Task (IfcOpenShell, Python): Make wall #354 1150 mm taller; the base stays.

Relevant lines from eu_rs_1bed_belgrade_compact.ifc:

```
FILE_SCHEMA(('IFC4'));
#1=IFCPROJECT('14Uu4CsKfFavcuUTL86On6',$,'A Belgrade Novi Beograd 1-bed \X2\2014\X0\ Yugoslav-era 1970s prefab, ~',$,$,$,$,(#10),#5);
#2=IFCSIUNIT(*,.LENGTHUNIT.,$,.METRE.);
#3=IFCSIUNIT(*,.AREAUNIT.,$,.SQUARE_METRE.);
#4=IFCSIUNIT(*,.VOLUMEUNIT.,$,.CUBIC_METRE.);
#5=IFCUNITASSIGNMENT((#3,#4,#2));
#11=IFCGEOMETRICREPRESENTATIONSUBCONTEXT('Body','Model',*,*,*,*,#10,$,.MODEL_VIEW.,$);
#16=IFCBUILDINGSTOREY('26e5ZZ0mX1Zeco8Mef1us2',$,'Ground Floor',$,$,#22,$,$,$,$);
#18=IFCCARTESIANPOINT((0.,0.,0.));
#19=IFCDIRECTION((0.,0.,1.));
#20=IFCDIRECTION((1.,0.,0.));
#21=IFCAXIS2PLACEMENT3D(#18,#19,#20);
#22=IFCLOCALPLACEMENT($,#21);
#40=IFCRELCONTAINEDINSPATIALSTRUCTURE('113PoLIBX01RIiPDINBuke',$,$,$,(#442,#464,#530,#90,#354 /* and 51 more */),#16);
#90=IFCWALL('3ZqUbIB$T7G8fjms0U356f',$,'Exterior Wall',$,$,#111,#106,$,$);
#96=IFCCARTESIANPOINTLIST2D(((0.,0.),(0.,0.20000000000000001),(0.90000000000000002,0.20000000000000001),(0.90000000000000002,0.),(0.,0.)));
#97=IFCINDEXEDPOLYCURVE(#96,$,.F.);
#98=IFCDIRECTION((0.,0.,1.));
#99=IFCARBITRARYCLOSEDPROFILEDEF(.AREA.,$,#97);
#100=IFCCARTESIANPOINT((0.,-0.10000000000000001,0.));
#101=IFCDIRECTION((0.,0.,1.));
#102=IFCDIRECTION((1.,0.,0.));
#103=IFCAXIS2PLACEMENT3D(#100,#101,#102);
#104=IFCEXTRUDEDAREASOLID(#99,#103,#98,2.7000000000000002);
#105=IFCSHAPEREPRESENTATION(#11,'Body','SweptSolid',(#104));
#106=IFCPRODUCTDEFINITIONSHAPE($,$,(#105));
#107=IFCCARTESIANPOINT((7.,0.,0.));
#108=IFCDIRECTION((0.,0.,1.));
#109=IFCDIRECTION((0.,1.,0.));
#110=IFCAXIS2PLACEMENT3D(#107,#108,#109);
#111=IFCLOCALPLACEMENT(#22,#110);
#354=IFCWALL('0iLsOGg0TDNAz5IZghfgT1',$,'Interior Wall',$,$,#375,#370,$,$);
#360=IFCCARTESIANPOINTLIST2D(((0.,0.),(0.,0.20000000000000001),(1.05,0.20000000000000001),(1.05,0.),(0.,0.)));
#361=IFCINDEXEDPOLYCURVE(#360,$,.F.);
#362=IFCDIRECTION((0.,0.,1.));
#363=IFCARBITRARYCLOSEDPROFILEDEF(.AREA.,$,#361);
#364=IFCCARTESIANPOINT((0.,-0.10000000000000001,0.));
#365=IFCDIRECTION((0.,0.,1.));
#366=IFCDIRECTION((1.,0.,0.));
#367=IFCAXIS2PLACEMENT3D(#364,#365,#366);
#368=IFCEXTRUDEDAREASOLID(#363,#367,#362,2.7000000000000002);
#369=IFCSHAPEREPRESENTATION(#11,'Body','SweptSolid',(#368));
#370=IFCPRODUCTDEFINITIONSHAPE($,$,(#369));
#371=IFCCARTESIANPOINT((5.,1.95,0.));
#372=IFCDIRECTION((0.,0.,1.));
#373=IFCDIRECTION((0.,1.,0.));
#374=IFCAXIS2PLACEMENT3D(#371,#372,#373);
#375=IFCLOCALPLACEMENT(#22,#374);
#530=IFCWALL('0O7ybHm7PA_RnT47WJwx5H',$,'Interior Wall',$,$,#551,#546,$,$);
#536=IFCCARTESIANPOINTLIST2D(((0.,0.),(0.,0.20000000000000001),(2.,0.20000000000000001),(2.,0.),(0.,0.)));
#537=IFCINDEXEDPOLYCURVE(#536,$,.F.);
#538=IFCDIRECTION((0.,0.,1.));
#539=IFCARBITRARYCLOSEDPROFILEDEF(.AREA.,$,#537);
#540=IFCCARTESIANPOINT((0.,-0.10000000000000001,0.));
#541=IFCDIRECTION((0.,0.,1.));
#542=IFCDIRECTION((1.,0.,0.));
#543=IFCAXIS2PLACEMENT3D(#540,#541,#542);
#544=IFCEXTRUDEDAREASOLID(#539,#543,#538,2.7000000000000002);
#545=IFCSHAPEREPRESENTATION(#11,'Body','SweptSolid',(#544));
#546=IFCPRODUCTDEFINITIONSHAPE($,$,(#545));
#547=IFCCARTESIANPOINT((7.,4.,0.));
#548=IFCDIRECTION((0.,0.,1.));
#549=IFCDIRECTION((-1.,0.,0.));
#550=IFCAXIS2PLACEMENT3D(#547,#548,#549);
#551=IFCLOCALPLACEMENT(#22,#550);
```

```python
import ifcopenshell
import ifcopenshell.geom
import ifcopenshell.util.representation
import ifcopenshell.util.shape

model = ifcopenshell.open("eu_rs_1bed_belgrade_compact.ifc")
settings = ifcopenshell.geom.settings()


def volume(element):
    """Net volume in cubic metres, openings subtracted."""
    shape = ifcopenshell.geom.create_shape(settings, element)
    return ifcopenshell.util.shape.get_volume(shape.geometry)


wall = model.by_guid("0iLsOGg0TDNAz5IZghfgT1")
before = volume(wall)

body = ifcopenshell.util.representation.get_representation(wall, "Model", "Body")
solid = body.Items[0]
old_height = solid.Depth
solid.Depth += 1.15
after = volume(wall)

print(f"height {old_height:g} -> {solid.Depth:g}, volume {before:.3f} -> {after:.3f} m3")

model.write("eu_rs_1bed_belgrade_compact-out.ifc")
```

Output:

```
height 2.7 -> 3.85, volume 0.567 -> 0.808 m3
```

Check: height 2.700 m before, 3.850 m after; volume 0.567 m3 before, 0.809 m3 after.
